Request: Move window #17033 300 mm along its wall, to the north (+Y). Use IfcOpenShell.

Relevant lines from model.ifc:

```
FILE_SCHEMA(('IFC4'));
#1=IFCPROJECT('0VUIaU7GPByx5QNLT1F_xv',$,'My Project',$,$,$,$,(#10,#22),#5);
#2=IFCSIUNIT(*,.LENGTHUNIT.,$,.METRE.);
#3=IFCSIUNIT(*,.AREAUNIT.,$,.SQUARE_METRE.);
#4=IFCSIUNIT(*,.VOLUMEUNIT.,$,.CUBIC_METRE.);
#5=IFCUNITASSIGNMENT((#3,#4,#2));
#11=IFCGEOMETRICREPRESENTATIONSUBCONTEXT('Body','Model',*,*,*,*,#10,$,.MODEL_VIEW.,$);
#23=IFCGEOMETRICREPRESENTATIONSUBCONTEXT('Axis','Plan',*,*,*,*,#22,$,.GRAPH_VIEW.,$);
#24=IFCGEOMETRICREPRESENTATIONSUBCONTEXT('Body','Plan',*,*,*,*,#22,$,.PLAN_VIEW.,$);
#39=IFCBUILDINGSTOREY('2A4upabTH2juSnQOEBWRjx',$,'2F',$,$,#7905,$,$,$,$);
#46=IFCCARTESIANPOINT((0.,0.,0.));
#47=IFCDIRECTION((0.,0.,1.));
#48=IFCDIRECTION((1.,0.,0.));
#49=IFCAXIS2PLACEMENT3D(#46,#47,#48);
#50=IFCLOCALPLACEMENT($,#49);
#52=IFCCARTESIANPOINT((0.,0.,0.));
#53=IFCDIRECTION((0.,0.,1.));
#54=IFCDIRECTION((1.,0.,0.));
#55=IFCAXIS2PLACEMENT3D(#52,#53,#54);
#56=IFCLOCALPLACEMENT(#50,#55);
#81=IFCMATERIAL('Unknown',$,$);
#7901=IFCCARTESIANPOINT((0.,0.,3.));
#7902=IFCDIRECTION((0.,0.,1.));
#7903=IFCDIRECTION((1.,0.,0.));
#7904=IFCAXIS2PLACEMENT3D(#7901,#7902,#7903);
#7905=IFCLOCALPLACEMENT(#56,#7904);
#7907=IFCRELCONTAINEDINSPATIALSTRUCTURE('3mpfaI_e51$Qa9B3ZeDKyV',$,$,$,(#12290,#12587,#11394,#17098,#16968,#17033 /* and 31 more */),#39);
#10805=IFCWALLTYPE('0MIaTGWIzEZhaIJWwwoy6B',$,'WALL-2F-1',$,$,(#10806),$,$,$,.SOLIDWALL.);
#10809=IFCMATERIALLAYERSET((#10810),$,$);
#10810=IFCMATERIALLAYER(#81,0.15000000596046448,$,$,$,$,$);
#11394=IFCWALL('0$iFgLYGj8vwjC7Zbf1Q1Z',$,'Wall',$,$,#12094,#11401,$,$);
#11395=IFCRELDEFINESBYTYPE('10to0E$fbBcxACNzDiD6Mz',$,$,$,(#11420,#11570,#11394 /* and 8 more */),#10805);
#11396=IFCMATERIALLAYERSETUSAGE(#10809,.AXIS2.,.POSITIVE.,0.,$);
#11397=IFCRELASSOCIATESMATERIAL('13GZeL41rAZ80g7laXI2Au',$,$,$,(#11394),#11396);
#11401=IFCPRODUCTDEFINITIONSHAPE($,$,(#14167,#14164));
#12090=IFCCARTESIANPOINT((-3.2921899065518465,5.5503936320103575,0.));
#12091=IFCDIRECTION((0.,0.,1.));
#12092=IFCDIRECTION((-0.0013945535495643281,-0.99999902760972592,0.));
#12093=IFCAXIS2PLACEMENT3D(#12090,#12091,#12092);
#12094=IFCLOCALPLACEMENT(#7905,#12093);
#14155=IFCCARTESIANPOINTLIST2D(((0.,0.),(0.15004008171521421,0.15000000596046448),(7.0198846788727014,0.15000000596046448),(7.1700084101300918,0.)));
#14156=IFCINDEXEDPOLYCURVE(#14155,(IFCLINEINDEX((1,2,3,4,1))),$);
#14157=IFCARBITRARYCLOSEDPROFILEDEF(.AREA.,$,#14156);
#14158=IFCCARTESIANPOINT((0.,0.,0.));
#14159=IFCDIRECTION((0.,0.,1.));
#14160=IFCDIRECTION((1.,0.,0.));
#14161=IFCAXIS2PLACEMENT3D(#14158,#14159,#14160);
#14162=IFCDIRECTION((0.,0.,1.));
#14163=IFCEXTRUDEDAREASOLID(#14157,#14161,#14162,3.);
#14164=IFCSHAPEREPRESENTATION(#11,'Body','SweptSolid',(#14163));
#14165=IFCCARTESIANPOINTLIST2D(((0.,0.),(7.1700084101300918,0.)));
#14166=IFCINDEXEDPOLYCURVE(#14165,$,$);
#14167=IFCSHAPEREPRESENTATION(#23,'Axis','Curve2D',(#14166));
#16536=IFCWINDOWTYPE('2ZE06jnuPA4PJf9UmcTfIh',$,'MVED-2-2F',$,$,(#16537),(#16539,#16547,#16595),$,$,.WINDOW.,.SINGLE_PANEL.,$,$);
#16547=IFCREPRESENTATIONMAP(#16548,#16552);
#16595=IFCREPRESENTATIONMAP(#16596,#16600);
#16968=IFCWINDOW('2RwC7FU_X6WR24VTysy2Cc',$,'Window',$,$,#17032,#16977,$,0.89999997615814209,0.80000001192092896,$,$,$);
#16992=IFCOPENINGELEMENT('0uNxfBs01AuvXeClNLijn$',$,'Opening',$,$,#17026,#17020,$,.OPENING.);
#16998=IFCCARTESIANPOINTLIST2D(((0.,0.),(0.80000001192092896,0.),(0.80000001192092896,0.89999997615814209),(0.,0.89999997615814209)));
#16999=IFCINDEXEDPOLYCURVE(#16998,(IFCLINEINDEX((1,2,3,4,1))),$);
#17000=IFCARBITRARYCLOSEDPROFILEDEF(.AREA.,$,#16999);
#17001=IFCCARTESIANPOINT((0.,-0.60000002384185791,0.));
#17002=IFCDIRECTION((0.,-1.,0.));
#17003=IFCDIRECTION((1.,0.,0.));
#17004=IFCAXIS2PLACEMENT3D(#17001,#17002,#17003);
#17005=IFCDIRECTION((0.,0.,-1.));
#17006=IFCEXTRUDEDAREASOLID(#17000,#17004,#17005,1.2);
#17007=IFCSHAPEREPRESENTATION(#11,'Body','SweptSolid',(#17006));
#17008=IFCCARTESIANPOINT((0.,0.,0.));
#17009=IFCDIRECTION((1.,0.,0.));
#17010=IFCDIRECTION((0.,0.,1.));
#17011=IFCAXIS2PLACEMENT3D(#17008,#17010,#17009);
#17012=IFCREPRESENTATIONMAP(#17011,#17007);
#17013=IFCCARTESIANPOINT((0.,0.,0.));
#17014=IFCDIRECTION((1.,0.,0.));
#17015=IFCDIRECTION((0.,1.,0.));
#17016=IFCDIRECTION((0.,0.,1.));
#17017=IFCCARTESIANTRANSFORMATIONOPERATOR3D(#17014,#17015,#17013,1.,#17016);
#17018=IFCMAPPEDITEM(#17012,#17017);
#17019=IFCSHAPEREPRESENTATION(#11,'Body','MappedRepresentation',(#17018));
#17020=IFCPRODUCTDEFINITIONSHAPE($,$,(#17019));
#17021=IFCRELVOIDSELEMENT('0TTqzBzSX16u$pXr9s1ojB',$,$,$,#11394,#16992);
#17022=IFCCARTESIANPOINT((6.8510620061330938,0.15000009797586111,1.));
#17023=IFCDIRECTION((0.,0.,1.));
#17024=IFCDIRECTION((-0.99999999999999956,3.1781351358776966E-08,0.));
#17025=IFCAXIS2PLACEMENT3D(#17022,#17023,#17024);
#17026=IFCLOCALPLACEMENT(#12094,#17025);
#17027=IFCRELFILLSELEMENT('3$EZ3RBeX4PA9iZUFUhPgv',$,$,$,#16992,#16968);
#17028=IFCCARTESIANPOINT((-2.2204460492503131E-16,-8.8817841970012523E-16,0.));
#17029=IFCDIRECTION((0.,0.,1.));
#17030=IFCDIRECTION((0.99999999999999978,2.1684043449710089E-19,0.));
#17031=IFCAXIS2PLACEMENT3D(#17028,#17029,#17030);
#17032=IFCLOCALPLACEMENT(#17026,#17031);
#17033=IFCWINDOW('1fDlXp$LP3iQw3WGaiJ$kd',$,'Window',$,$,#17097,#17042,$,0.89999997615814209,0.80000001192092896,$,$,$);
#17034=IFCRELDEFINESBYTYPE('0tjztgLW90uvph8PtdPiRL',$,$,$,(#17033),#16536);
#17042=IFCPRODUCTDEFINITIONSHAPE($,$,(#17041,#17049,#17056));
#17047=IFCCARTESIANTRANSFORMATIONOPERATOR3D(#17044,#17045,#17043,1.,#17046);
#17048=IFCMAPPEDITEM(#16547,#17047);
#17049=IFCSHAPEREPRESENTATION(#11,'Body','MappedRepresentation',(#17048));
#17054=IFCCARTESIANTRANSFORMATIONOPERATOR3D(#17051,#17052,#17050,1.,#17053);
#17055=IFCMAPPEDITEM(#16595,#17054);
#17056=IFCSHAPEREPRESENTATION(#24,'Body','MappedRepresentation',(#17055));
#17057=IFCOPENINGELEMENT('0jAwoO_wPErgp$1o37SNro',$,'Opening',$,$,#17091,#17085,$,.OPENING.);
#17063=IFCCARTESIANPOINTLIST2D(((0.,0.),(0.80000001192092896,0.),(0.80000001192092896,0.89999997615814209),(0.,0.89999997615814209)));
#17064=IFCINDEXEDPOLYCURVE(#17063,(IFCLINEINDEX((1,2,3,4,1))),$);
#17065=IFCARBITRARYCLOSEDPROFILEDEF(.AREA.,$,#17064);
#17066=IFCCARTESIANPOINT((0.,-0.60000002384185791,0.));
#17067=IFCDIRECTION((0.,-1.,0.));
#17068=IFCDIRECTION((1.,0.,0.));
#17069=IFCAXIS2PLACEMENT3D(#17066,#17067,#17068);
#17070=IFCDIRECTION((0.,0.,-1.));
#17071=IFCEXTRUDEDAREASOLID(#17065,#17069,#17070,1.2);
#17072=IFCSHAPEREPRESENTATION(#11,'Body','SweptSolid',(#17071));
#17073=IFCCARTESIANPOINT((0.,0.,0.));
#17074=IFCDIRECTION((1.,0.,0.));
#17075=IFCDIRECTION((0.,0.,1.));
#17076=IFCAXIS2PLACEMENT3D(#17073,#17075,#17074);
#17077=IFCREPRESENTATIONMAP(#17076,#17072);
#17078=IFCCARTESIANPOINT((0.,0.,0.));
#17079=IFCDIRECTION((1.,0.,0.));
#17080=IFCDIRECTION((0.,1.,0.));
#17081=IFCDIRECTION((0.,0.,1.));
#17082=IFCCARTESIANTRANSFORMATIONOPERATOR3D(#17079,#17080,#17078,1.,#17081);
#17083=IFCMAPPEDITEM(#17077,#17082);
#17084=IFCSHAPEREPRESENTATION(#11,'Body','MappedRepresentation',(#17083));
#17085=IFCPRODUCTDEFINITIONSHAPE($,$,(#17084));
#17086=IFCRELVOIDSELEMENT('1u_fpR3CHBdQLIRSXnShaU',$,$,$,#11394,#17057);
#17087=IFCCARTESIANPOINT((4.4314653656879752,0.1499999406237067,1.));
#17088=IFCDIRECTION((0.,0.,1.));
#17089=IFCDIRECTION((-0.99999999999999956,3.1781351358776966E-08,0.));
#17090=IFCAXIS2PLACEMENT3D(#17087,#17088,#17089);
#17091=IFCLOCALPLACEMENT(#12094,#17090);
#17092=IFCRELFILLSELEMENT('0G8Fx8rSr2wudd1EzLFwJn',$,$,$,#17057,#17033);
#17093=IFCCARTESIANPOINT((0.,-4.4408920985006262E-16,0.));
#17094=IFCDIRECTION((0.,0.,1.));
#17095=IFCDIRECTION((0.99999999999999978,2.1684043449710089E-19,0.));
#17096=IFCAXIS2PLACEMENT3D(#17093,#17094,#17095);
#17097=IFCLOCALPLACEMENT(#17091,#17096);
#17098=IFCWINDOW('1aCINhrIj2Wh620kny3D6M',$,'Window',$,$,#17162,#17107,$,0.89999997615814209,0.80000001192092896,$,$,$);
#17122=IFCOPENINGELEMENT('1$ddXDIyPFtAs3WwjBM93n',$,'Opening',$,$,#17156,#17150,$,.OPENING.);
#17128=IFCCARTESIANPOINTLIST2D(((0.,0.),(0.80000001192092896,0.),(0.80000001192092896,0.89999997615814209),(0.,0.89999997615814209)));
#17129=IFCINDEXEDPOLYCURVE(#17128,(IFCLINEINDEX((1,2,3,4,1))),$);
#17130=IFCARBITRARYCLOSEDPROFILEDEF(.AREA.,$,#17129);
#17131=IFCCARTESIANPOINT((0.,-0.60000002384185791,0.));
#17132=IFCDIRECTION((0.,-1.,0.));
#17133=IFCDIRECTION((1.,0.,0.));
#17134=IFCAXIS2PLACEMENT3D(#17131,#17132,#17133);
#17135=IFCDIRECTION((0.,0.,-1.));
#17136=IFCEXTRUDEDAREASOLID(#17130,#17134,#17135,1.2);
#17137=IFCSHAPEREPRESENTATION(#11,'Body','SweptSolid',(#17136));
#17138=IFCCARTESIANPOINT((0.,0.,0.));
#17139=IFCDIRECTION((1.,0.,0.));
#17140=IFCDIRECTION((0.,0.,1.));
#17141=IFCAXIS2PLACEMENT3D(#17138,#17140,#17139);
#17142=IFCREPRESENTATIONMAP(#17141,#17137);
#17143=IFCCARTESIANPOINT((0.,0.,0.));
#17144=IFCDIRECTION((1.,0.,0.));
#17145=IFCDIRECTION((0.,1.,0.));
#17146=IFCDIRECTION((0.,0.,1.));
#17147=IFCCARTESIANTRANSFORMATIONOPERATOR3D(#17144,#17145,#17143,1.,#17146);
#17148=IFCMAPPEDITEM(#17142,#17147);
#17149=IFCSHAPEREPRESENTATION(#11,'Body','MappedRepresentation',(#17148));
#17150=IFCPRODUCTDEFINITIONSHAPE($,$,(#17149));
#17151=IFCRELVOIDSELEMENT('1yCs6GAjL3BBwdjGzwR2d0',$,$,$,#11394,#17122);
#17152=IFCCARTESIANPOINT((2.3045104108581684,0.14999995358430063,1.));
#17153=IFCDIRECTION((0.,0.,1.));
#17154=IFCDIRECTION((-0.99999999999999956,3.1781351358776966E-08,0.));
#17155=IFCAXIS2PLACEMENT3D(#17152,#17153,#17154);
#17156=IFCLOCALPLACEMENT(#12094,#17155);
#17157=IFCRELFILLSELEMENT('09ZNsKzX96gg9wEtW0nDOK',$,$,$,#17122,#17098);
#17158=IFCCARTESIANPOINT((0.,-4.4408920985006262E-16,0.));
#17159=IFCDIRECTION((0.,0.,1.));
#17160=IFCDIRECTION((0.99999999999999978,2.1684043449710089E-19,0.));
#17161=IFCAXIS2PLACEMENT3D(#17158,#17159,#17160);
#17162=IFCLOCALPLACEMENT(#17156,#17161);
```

```python
import ifcopenshell
import ifcopenshell.api.geometry
import ifcopenshell.util.placement
import ifcopenshell.util.unit

model = ifcopenshell.open("model.ifc")
unit_scale = ifcopenshell.util.unit.calculate_unit_scale(model)

window = model.by_guid("1fDlXp$LP3iQw3WGaiJ$kd")
opening = window.FillsVoids[0].RelatingOpeningElement
wall = opening.VoidsElements[0].RelatingBuildingElement

wall_matrix = ifcopenshell.util.placement.get_local_placement(wall.ObjectPlacement)
shift = wall_matrix[:3, 0] * -0.3 / unit_scale
before = ifcopenshell.util.placement.get_local_placement(window.ObjectPlacement)[:3, 3].copy()

# The window is placed relative to its opening, so it follows when the opening moves.
matrix = ifcopenshell.util.placement.get_local_placement(opening.ObjectPlacement)
matrix[:3, 3] += shift
ifcopenshell.api.geometry.edit_object_placement(
    model, product=opening, matrix=matrix, is_si=False, should_transform_children=True
)

after = ifcopenshell.util.placement.get_local_placement(window.ObjectPlacement)[:3, 3]
print("window moved by", (after - before).round(3) + 0.0)

model.write("model_v2.ifc")
```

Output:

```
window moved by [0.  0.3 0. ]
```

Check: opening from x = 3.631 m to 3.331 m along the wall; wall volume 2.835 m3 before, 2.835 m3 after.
